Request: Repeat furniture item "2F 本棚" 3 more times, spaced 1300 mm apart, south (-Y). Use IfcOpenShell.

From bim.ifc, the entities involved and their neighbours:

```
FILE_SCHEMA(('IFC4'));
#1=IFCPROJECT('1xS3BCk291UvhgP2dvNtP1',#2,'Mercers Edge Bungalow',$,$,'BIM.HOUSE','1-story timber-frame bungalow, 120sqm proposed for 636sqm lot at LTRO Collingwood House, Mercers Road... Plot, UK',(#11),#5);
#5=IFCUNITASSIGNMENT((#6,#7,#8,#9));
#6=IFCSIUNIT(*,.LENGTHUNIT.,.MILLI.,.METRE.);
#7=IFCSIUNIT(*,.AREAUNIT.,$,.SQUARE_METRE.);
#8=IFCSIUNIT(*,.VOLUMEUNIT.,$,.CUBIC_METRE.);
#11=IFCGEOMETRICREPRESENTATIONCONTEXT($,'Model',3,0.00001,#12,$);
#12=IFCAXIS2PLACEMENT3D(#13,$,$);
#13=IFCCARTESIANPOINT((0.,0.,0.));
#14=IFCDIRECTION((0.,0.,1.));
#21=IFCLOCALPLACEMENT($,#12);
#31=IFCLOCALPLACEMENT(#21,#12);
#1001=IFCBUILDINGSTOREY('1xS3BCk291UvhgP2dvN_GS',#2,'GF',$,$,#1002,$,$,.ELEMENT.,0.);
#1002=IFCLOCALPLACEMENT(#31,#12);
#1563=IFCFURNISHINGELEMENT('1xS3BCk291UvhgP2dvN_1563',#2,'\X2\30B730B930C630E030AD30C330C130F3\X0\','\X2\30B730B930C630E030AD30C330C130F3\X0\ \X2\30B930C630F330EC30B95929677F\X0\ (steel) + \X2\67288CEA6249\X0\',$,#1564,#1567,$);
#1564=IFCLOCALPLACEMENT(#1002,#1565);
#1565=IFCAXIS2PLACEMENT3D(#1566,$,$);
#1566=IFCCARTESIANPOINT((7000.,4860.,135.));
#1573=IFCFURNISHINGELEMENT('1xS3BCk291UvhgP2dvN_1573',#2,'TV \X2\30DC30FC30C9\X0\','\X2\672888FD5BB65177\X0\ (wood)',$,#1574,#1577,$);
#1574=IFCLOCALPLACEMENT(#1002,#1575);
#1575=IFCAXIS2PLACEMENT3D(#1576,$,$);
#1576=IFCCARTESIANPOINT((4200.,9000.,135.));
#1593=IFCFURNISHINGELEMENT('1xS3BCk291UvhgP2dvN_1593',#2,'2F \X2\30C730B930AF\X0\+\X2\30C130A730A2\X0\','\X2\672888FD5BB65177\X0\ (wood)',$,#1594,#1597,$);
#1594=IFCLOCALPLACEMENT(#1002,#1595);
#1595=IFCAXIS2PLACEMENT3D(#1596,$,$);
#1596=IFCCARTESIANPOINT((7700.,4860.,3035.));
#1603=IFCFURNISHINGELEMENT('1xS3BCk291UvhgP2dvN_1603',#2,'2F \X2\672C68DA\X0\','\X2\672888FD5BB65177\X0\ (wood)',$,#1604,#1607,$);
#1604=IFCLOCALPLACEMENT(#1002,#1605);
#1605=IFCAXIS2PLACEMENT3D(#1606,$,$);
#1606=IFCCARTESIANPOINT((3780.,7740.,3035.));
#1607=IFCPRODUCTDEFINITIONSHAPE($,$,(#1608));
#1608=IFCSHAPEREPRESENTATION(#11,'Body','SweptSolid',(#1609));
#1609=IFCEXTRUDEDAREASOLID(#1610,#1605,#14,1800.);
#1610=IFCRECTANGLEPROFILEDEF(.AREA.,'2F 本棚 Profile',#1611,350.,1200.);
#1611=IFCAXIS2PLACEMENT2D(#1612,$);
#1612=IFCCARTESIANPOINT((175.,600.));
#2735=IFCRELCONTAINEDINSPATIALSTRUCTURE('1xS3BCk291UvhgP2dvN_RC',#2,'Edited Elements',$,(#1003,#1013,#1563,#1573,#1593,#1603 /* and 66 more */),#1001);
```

```python
import numpy as np
import ifcopenshell
import ifcopenshell.api.geometry
import ifcopenshell.api.root
import ifcopenshell.util.element
import ifcopenshell.util.placement

model = ifcopenshell.open("bim.ifc")


def reuse_history(source, copy):
    """copy_class also copies each property set's owner history, people and application; keep the originals."""
    for rel in copy.IsDefinedBy:
        if rel.is_a("IfcRelDefinesByProperties") and (history := rel.RelatingPropertyDefinition.OwnerHistory):
            rel.RelatingPropertyDefinition.OwnerHistory = source.OwnerHistory
            ifcopenshell.util.element.remove_deep2(model, history)


source = model.by_guid("1xS3BCk291UvhgP2dvN_1603")
base = ifcopenshell.util.placement.get_local_placement(source.ObjectPlacement)
step = np.array([0.0, -1.0, 0.0]) * 1300.0

for i in range(1, 4):
    copy = ifcopenshell.api.root.copy_class(model, product=source)
    copy.Representation = ifcopenshell.util.element.copy_deep(
        model, source.Representation, exclude=["IfcGeometricRepresentationContext", "IfcRepresentationMap"]
    )
    reuse_history(source, copy)
    matrix = base.copy()
    matrix[:3, 3] += i * step
    print("added at", matrix[:3, 3].round(3) + 0.0)
    ifcopenshell.api.geometry.edit_object_placement(model, product=copy, matrix=matrix, is_si=False)

model.write("bim-out.ifc")
```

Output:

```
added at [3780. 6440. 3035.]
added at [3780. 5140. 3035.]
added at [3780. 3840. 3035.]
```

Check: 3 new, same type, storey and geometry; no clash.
